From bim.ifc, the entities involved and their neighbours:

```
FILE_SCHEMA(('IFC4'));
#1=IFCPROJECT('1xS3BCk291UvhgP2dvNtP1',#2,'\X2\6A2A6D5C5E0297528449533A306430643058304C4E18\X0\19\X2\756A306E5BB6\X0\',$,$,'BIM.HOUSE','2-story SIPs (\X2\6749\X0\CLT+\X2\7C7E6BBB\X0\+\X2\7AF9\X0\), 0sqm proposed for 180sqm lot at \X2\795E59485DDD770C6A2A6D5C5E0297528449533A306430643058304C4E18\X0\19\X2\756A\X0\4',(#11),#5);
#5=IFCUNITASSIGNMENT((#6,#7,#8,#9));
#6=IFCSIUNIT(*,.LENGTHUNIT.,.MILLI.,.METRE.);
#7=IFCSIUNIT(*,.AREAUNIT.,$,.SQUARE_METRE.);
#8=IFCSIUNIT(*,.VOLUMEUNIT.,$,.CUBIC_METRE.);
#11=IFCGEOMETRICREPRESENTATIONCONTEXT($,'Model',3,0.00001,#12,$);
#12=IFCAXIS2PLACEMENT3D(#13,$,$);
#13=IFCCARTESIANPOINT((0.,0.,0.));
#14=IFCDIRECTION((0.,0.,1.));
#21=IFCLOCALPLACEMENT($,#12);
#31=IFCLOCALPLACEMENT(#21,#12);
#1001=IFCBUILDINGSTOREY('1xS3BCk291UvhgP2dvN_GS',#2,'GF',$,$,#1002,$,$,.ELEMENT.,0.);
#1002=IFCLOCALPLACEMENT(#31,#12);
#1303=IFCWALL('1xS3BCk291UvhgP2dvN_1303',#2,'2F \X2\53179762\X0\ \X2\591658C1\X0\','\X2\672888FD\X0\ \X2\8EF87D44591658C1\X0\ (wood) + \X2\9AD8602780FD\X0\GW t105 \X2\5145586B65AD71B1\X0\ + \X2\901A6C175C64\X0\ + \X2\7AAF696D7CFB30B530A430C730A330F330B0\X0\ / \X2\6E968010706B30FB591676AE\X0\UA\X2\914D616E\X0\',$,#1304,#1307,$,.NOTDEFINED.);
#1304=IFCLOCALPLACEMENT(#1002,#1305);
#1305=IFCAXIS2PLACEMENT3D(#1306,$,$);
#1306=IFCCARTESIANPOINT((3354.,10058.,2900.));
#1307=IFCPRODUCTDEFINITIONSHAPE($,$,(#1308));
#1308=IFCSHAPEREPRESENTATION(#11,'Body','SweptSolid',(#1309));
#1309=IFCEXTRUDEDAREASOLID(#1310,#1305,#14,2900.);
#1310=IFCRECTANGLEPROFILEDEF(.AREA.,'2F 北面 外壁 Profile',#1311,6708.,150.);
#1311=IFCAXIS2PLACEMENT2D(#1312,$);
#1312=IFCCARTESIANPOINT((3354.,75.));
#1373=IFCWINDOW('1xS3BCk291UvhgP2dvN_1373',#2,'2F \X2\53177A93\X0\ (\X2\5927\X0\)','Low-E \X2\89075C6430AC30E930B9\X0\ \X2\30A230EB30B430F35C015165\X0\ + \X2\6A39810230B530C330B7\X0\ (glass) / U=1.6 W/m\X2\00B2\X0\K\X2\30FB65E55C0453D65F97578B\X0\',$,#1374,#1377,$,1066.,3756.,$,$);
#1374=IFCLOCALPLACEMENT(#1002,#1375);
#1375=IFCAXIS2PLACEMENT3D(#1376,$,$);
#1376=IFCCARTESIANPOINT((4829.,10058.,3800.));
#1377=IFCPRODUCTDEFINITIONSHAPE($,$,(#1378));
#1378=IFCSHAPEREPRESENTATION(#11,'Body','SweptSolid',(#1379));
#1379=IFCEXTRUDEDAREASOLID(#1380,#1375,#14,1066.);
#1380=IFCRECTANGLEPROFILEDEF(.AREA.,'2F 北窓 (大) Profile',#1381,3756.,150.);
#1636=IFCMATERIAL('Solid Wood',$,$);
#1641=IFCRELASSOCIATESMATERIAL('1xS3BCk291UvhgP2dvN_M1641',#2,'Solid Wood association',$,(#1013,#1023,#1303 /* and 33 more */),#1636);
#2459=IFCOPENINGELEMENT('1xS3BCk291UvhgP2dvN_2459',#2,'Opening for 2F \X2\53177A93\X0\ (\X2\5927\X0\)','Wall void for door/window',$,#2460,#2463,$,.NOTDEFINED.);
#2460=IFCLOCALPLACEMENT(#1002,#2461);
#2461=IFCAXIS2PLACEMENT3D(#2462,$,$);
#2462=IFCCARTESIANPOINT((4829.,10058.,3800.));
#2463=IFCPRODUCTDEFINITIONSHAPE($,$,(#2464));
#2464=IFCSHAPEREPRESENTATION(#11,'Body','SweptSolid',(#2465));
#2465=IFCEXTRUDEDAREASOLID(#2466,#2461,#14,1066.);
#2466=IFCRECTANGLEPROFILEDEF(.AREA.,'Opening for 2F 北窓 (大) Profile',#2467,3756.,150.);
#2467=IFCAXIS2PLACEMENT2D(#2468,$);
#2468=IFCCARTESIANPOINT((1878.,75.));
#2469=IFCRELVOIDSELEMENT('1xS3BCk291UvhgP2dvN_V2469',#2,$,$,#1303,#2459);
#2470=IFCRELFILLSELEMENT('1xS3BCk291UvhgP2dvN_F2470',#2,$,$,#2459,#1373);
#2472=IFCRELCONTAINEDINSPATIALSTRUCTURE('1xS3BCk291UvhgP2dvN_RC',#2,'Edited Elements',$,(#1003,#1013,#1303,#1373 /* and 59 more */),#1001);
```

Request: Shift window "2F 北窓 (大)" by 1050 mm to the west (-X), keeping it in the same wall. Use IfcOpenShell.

```python
import ifcopenshell
import ifcopenshell.api.geometry
import ifcopenshell.util.placement
import ifcopenshell.util.unit

model = ifcopenshell.open("bim.ifc")
unit_scale = ifcopenshell.util.unit.calculate_unit_scale(model)

window = model.by_guid("1xS3BCk291UvhgP2dvN_1373")
opening = window.FillsVoids[0].RelatingOpeningElement
wall = opening.VoidsElements[0].RelatingBuildingElement

wall_matrix = ifcopenshell.util.placement.get_local_placement(wall.ObjectPlacement)
shift = wall_matrix[:3, 0] * -1.05 / unit_scale
before = ifcopenshell.util.placement.get_local_placement(window.ObjectPlacement)[:3, 3].copy()

# The window is not placed relative to its opening, so move both.
for product in (opening, window):
    matrix = ifcopenshell.util.placement.get_local_placement(product.ObjectPlacement)
    matrix[:3, 3] += shift
    ifcopenshell.api.geometry.edit_object_placement(model, product=product, matrix=matrix, is_si=False)

after = ifcopenshell.util.placement.get_local_placement(window.ObjectPlacement)[:3, 3]
print("window moved by", (after - before).round(3) + 0.0)

model.write("bim_updated.ifc")
```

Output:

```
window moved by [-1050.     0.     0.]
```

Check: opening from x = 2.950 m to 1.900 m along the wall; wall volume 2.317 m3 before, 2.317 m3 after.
